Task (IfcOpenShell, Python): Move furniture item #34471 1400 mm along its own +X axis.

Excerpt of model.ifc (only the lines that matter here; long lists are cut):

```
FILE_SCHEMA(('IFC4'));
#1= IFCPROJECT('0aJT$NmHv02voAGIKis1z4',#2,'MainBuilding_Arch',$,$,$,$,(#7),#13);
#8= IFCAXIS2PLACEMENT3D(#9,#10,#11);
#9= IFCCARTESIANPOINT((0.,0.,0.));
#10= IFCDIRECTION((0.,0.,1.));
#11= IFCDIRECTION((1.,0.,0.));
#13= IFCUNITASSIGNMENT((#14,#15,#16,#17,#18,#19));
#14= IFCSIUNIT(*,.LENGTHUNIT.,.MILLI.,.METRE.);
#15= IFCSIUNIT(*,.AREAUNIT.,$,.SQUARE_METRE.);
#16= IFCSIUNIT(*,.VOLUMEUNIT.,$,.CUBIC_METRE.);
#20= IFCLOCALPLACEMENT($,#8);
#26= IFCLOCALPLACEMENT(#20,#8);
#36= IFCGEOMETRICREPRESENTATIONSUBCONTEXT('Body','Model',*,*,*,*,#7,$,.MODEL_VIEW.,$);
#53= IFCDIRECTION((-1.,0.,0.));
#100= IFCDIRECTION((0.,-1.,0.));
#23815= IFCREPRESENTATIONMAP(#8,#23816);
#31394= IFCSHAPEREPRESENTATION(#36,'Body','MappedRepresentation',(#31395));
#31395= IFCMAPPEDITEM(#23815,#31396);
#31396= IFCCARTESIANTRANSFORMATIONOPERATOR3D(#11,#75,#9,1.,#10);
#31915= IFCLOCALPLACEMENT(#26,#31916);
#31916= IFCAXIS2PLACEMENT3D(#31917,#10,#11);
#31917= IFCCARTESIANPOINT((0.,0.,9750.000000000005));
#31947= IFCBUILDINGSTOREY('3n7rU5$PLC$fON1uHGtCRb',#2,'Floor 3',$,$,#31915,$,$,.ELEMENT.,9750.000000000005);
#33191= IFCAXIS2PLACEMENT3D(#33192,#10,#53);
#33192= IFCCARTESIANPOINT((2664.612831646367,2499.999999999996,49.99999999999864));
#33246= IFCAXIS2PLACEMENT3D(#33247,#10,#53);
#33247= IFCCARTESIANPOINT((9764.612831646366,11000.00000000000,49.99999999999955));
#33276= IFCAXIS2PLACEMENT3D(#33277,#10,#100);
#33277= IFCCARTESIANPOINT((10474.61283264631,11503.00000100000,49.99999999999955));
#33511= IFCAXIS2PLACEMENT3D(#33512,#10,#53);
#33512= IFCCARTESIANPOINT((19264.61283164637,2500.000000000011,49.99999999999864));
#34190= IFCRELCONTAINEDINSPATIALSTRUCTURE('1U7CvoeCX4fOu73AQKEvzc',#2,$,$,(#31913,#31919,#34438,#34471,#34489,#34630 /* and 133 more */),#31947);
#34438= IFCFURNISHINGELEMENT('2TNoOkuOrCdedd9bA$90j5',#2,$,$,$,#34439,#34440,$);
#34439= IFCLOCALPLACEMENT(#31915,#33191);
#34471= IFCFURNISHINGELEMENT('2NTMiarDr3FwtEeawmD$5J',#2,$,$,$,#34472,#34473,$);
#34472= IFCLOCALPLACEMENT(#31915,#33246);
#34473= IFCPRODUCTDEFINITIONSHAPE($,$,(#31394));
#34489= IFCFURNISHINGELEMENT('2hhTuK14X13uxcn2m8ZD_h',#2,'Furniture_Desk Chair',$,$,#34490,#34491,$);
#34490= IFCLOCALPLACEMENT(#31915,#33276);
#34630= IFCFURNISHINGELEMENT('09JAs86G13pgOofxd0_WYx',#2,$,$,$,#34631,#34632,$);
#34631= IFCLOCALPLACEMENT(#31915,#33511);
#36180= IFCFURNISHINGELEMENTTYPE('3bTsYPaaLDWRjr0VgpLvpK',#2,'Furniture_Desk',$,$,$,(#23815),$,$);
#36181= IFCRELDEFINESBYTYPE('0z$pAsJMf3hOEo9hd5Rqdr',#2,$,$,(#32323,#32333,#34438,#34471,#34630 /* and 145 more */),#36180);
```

```python
import ifcopenshell
import ifcopenshell.api.geometry
import ifcopenshell.util.placement

model = ifcopenshell.open("model.ifc")

item = model.by_guid("2NTMiarDr3FwtEeawmD$5J")
matrix = ifcopenshell.util.placement.get_local_placement(item.ObjectPlacement)
matrix[:3, 3] += matrix[:3, 0] * 1400.0
ifcopenshell.api.geometry.edit_object_placement(model, product=item, matrix=matrix, is_si=False)

print(ifcopenshell.util.placement.get_local_placement(item.ObjectPlacement).round(3) + 0.0)

model.write("model_updated.ifc")
```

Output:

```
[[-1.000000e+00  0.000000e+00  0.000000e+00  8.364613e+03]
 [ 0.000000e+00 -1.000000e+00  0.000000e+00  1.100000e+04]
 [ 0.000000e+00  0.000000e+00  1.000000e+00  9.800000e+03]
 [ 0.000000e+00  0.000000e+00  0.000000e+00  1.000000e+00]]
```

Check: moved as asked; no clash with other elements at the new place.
